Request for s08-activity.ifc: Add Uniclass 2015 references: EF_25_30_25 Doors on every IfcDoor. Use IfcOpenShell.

First a look at what the model holds.

```python
import ifcopenshell

model = ifcopenshell.open("s08-activity.ifc")
print(model.schema)
print("classifications:", [c.Name for c in model.by_type("IfcClassification")])
for ifc_class in ("IfcDoor", "IfcRoof", "IfcStair", "IfcWall", "IfcWindow"):
    print(ifc_class, len(model.by_type(ifc_class)))
```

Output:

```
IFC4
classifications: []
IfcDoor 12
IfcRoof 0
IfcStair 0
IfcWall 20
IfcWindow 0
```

```python
import ifcopenshell
import ifcopenshell.api.classification

model = ifcopenshell.open("s08-activity.ifc")

system = ifcopenshell.api.classification.add_classification(model, classification="Uniclass 2015")

codes = {
    "IfcDoor": ("EF_25_30_25", "Doors"),
}
for ifc_class, (code, name) in codes.items():
    products = model.by_type(ifc_class)
    ifcopenshell.api.classification.add_reference(
        model, products=products, classification=system, identification=code, name=name
    )
    print(code, len(products))

model.write("s08-activity_v2.ifc")
```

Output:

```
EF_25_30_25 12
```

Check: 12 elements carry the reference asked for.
